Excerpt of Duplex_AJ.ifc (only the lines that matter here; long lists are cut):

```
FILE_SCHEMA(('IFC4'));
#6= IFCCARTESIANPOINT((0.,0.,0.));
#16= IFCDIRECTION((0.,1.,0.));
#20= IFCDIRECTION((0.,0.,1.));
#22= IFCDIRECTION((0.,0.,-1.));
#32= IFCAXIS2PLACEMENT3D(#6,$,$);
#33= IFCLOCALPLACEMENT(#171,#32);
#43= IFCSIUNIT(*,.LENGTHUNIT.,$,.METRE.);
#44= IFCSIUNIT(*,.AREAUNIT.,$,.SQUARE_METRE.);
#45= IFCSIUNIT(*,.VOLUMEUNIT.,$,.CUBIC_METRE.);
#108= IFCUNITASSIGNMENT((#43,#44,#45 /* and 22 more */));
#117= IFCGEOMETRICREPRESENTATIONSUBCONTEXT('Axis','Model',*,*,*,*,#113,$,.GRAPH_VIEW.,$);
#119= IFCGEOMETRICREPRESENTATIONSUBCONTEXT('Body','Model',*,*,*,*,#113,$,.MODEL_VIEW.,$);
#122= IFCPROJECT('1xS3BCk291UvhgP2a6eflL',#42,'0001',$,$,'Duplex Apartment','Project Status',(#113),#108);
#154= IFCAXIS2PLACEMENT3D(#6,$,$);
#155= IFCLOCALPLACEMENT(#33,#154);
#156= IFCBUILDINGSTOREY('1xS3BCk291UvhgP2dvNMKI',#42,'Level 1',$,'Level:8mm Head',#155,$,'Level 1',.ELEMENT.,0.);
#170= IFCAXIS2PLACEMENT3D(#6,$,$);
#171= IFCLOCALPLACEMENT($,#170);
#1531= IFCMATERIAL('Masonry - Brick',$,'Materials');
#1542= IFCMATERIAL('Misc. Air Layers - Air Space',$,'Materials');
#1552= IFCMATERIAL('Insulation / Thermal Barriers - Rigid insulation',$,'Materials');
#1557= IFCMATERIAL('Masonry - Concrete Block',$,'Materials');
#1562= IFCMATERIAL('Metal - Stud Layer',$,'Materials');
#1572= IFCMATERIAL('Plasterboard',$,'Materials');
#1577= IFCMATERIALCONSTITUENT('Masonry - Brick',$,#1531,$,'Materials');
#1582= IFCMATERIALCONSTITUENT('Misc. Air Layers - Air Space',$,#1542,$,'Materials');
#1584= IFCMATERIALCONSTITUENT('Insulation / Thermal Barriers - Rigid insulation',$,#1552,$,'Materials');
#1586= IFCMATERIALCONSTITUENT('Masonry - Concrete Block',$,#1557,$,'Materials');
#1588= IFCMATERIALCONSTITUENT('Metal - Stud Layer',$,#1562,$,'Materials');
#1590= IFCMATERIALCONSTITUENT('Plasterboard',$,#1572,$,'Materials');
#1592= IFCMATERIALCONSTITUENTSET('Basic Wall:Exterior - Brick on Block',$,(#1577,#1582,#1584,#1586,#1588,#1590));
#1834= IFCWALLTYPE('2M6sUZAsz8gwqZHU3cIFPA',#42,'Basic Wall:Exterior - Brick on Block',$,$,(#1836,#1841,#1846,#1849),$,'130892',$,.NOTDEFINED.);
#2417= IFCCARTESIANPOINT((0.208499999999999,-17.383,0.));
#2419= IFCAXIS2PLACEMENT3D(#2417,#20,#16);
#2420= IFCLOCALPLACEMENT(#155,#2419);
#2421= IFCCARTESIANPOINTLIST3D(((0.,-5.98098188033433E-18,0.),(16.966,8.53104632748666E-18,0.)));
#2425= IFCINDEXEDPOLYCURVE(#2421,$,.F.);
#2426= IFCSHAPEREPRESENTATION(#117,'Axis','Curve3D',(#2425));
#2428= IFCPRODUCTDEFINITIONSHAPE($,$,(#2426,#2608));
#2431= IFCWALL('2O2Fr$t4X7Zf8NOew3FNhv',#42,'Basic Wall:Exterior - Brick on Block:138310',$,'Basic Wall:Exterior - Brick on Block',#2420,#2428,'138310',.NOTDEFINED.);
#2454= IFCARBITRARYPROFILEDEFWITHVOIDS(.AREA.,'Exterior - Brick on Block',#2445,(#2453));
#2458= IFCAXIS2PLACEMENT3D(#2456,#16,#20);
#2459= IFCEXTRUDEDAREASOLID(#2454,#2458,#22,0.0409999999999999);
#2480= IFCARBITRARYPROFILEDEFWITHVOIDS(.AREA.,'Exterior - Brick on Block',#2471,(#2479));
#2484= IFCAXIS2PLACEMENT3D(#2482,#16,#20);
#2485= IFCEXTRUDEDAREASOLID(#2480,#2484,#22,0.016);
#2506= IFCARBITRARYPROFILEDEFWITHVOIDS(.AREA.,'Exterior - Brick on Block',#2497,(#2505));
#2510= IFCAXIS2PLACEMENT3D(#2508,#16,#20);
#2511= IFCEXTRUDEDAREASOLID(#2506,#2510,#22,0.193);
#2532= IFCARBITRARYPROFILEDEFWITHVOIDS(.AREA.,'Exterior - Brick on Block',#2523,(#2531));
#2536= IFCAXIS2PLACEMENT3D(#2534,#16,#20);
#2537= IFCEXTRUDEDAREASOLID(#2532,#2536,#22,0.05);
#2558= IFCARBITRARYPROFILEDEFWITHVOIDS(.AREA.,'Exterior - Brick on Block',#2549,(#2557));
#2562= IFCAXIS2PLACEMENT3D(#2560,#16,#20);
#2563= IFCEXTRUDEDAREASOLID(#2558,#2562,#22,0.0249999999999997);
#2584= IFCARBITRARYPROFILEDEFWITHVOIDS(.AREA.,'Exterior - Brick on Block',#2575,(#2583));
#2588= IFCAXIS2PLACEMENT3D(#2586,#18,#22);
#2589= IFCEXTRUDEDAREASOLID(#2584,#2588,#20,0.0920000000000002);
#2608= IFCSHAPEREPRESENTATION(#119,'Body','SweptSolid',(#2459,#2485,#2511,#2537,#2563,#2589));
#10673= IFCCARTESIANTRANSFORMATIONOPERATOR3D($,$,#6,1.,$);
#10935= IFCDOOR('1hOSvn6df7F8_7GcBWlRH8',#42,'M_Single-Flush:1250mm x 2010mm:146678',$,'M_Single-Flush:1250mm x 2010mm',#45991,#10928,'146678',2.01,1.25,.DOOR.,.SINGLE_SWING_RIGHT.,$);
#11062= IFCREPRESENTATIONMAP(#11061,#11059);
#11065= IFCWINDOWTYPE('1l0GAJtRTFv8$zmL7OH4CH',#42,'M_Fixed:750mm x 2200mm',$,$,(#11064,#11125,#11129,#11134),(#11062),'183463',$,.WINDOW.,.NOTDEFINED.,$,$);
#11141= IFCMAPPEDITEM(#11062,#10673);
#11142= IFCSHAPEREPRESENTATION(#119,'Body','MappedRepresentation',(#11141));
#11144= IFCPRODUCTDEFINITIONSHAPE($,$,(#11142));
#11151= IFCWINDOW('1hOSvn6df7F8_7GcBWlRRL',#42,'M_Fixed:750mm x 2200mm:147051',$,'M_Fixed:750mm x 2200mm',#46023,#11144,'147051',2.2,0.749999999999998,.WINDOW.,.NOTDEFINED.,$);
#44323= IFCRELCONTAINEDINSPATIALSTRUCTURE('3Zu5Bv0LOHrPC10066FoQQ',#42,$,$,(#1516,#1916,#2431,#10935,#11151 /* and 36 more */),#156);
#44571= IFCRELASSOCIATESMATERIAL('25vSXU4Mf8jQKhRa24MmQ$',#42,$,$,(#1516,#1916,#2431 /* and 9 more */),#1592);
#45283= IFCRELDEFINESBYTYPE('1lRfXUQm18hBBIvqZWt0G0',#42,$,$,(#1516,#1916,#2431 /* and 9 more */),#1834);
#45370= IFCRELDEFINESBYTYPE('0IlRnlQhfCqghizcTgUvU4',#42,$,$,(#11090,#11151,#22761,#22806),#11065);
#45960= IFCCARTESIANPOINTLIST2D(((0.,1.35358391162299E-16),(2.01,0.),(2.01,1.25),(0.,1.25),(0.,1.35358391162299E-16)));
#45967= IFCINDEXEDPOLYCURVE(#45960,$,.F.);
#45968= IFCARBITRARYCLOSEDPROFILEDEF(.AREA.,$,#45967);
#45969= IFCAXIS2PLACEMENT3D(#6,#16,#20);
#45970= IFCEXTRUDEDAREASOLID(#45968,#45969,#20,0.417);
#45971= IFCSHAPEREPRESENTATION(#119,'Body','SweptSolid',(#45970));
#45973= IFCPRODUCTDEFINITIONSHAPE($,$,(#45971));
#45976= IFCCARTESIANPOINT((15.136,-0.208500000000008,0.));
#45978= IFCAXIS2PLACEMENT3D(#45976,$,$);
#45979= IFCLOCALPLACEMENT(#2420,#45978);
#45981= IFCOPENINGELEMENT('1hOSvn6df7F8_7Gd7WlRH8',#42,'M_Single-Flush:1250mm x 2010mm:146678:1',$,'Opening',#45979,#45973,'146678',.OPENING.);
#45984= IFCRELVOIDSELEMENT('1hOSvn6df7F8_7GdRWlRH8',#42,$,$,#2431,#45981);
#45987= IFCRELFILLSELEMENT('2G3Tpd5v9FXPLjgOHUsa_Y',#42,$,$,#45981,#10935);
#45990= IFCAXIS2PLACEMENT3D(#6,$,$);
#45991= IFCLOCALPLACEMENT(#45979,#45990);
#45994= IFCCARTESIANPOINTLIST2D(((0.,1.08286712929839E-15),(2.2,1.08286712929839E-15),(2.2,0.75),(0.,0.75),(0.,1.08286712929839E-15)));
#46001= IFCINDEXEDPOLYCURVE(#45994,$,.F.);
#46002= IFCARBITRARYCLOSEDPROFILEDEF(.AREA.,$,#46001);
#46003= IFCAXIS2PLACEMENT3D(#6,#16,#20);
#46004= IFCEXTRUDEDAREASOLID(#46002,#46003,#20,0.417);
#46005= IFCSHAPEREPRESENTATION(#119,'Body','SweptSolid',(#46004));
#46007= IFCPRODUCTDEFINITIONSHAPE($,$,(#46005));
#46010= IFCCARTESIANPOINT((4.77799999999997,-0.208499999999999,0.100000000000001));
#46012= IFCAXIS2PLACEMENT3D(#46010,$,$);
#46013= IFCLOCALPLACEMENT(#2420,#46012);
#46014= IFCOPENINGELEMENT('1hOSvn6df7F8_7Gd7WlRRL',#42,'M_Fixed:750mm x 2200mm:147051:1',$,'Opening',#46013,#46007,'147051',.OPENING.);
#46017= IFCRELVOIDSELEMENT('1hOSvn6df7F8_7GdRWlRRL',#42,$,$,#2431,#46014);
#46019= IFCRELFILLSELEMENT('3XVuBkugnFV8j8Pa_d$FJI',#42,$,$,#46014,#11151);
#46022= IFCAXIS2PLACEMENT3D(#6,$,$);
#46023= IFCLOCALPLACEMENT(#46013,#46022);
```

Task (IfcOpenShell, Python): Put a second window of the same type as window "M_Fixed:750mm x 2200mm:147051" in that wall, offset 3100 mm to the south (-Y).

```python
import ifcopenshell
import ifcopenshell.api.feature
import ifcopenshell.api.geometry
import ifcopenshell.api.root
import ifcopenshell.geom
import ifcopenshell.util.element
import ifcopenshell.util.placement
import ifcopenshell.util.shape

model = ifcopenshell.open("Duplex_AJ.ifc")
settings = ifcopenshell.geom.settings()


def volume(element):
    """Net volume in cubic metres, openings subtracted."""
    shape = ifcopenshell.geom.create_shape(settings, element)
    return ifcopenshell.util.shape.get_volume(shape.geometry)


def reuse_history(source, copy):
    """copy_class also copies each property set's owner history, people and application; keep the originals."""
    for rel in copy.IsDefinedBy:
        if rel.is_a("IfcRelDefinesByProperties") and (history := rel.RelatingPropertyDefinition.OwnerHistory):
            rel.RelatingPropertyDefinition.OwnerHistory = source.OwnerHistory
            ifcopenshell.util.element.remove_deep2(model, history)


window = model.by_guid("1hOSvn6df7F8_7GcBWlRRL")
opening = window.FillsVoids[0].RelatingOpeningElement
wall = opening.VoidsElements[0].RelatingBuildingElement
before = volume(wall)
shift = ifcopenshell.util.placement.get_local_placement(wall.ObjectPlacement)[:3, 0] * -3.1

# copy_class copies the void relationship, type, container and properties, but no geometry.
new_opening = ifcopenshell.api.root.copy_class(model, product=opening)
new_opening.Representation = ifcopenshell.util.element.copy_deep(
    model, opening.Representation, exclude=["IfcGeometricRepresentationContext", "IfcRepresentationMap"]
)
new_opening.Name = "M_Fixed:750mm x 2200mm"
new_opening.Tag = None
new_window = ifcopenshell.api.root.copy_class(model, product=window)
new_window.Representation = ifcopenshell.util.element.copy_deep(
    model, window.Representation, exclude=["IfcGeometricRepresentationContext", "IfcRepresentationMap"]
)
new_window.Name = "M_Fixed:750mm x 2200mm"
new_window.Tag = None
reuse_history(window, new_window)
ifcopenshell.api.feature.add_filling(model, opening=new_opening, element=new_window)

for old, new in ((opening, new_opening), (window, new_window)):
    matrix = ifcopenshell.util.placement.get_local_placement(old.ObjectPlacement)
    matrix[:3, 3] += shift
    ifcopenshell.api.geometry.edit_object_placement(model, product=new, matrix=matrix, is_si=False)

after = volume(wall)

print(f"wall volume {before:.3f} -> {after:.3f} m3")

model.write("Duplex_AJ_edited.ifc")
```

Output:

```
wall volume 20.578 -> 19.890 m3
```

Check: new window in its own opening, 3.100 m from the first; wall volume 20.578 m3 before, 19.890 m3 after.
